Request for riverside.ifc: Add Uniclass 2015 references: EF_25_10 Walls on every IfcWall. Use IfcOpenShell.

First a look at what the model holds.

```python
import ifcopenshell

model = ifcopenshell.open("riverside.ifc")
print(model.schema)
print("classifications:", [c.Name for c in model.by_type("IfcClassification")])
for ifc_class in ("IfcDoor", "IfcRoof", "IfcStair", "IfcWall", "IfcWindow"):
    print(ifc_class, len(model.by_type(ifc_class)))
```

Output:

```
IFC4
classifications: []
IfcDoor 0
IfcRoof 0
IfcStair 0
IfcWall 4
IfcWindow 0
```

```python
import ifcopenshell
import ifcopenshell.api.classification

model = ifcopenshell.open("riverside.ifc")

system = ifcopenshell.api.classification.add_classification(model, classification="Uniclass 2015")

codes = {
    "IfcWall": ("EF_25_10", "Walls"),
}
for ifc_class, (code, name) in codes.items():
    products = model.by_type(ifc_class)
    ifcopenshell.api.classification.add_reference(
        model, products=products, classification=system, identification=code, name=name
    )
    print(code, len(products))

model.write("riverside_v2.ifc")
```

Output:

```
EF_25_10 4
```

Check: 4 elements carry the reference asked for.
